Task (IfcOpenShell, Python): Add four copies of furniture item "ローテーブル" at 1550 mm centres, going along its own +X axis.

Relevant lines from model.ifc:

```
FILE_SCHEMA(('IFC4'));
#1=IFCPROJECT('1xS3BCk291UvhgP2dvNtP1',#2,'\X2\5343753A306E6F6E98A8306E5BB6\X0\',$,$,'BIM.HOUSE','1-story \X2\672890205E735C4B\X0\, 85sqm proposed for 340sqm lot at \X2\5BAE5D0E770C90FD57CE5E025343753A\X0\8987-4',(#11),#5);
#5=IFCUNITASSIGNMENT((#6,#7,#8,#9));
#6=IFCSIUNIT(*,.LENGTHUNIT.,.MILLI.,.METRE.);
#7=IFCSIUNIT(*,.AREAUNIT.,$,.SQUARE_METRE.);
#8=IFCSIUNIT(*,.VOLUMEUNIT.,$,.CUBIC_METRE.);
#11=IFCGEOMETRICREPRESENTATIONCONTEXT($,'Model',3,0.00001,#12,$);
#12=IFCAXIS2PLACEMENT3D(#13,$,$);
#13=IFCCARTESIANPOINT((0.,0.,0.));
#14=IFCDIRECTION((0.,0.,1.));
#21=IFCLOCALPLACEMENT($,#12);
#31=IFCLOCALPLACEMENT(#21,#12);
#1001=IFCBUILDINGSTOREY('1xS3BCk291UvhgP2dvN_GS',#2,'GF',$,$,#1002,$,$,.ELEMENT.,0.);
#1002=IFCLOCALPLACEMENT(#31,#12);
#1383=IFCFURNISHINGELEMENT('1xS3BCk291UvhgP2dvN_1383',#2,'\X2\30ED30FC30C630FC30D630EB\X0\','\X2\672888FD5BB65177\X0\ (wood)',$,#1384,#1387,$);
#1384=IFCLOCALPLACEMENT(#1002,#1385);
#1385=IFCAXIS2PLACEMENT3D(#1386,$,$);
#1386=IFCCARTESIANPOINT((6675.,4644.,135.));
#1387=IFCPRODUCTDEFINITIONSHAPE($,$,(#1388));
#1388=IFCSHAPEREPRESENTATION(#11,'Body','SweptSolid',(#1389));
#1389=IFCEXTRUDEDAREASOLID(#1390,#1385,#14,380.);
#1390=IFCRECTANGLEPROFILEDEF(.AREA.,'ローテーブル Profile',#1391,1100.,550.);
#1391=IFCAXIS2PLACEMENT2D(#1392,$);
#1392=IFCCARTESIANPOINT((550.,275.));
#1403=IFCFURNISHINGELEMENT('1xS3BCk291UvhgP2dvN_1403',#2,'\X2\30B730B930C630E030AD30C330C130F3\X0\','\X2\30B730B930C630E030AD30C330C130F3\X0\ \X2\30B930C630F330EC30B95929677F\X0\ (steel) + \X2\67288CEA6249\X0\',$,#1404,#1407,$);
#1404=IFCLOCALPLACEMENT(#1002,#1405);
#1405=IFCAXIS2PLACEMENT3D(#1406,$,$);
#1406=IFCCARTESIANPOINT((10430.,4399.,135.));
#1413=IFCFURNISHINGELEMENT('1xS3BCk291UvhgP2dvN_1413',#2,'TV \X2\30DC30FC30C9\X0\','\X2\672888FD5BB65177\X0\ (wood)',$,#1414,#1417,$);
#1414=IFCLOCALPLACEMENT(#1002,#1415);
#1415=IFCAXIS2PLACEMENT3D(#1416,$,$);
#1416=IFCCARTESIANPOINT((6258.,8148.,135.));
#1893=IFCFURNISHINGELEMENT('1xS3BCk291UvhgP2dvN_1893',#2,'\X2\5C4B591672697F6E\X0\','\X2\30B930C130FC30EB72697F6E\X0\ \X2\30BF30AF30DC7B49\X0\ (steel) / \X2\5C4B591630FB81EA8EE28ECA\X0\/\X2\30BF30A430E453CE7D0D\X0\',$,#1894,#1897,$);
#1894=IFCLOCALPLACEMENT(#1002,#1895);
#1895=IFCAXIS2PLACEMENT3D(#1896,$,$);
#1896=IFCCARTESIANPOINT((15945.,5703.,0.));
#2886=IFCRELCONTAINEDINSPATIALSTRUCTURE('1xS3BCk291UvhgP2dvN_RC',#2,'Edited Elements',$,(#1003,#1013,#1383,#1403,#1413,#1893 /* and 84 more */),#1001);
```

```python
import ifcopenshell
import ifcopenshell.api.geometry
import ifcopenshell.api.root
import ifcopenshell.util.element
import ifcopenshell.util.placement

model = ifcopenshell.open("model.ifc")


def reuse_history(source, copy):
    """copy_class also copies each property set's owner history, people and application; keep the originals."""
    for rel in copy.IsDefinedBy:
        if rel.is_a("IfcRelDefinesByProperties") and (history := rel.RelatingPropertyDefinition.OwnerHistory):
            rel.RelatingPropertyDefinition.OwnerHistory = source.OwnerHistory
            ifcopenshell.util.element.remove_deep2(model, history)


source = model.by_id(1383)
base = ifcopenshell.util.placement.get_local_placement(source.ObjectPlacement)
step = base[:3, 0] * 1550.0

for i in range(1, 5):
    copy = ifcopenshell.api.root.copy_class(model, product=source)
    copy.Representation = ifcopenshell.util.element.copy_deep(
        model, source.Representation, exclude=["IfcGeometricRepresentationContext", "IfcRepresentationMap"]
    )
    reuse_history(source, copy)
    matrix = base.copy()
    matrix[:3, 3] += i * step
    print("added at", matrix[:3, 3].round(3) + 0.0)
    ifcopenshell.api.geometry.edit_object_placement(model, product=copy, matrix=matrix, is_si=False)

model.write("model-out.ifc")
```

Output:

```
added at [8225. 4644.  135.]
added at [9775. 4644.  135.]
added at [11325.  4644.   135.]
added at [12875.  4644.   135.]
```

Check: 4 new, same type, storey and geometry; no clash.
